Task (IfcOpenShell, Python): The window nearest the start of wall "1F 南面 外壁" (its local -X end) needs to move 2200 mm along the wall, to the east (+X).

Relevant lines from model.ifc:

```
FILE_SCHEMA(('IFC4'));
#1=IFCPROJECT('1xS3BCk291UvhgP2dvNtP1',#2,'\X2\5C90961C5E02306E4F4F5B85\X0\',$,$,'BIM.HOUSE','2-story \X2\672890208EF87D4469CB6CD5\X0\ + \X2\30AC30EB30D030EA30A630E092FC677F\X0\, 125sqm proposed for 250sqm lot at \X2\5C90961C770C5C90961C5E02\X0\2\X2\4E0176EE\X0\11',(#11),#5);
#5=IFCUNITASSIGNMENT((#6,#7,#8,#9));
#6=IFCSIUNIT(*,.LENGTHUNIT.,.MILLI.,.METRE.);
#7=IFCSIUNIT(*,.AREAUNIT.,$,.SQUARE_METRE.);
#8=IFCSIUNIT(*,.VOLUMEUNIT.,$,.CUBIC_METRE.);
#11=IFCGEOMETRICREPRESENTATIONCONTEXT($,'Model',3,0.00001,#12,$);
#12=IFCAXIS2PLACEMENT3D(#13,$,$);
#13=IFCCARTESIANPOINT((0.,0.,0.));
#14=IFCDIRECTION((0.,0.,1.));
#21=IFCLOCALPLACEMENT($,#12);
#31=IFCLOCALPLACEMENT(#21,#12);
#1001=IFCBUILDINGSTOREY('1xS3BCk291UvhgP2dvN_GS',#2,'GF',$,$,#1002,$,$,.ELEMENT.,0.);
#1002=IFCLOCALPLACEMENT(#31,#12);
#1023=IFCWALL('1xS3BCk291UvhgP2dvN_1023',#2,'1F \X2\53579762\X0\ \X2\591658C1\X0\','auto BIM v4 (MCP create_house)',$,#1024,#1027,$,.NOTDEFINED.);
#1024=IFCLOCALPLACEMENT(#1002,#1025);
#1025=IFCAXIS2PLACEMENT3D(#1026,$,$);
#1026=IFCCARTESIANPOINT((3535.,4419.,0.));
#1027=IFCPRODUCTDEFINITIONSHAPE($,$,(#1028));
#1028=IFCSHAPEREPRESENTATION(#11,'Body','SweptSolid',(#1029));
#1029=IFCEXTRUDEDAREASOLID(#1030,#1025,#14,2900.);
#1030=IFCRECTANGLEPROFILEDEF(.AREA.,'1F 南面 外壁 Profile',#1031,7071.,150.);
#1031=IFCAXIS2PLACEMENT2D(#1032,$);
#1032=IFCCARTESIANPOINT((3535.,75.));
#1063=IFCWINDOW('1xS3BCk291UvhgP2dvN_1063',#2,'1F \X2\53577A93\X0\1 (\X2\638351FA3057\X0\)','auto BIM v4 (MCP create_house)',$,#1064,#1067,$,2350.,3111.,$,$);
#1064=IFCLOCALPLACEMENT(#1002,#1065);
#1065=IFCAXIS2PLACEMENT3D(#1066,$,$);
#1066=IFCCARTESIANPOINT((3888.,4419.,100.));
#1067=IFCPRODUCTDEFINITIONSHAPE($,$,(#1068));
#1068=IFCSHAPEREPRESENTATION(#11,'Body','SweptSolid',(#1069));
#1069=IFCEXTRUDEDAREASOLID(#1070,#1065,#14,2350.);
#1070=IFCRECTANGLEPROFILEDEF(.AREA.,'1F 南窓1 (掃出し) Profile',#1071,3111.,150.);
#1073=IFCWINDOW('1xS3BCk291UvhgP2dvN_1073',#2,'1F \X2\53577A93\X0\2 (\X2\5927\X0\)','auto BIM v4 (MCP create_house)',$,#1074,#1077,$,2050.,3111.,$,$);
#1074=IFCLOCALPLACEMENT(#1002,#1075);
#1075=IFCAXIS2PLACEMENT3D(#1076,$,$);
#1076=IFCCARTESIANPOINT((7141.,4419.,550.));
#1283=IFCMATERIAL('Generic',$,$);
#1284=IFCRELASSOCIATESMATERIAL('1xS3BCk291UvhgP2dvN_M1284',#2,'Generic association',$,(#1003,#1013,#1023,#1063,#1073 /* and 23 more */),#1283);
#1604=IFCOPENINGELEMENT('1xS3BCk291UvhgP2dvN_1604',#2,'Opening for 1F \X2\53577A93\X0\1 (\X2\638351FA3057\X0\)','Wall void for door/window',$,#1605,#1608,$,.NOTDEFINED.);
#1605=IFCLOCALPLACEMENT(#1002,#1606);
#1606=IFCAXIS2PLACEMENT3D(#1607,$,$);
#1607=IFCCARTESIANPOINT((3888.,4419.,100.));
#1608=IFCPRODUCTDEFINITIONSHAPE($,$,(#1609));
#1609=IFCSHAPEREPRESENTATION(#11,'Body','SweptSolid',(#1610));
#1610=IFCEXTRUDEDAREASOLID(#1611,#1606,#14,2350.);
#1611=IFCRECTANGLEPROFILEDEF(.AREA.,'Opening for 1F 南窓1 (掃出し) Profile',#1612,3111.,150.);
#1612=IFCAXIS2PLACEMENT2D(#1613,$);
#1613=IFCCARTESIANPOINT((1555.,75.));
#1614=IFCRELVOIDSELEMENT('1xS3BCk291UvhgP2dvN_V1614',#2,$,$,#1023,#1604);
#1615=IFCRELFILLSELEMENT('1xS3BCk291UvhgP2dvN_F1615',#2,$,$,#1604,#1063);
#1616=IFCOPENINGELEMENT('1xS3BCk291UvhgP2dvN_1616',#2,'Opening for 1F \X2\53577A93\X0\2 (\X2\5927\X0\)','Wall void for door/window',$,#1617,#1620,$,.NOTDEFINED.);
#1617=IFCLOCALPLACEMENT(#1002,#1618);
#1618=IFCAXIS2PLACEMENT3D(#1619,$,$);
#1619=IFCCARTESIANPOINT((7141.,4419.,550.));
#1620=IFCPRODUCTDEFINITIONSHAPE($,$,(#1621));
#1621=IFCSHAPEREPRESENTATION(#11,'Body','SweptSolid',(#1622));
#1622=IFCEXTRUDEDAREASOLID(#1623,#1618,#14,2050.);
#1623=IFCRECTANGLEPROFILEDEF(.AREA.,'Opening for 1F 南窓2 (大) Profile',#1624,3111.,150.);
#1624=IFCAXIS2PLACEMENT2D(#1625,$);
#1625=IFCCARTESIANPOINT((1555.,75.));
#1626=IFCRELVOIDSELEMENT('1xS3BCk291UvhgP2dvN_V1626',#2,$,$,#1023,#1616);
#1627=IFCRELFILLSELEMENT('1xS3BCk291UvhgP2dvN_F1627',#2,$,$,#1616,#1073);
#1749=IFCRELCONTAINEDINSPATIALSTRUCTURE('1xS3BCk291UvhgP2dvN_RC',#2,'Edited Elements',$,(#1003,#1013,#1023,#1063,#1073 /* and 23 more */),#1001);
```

```python
import ifcopenshell
import ifcopenshell.api.geometry
import ifcopenshell.util.placement
import ifcopenshell.util.unit

model = ifcopenshell.open("model.ifc")
unit_scale = ifcopenshell.util.unit.calculate_unit_scale(model)

window = model.by_guid("1xS3BCk291UvhgP2dvN_1063")
opening = window.FillsVoids[0].RelatingOpeningElement
wall = opening.VoidsElements[0].RelatingBuildingElement

wall_matrix = ifcopenshell.util.placement.get_local_placement(wall.ObjectPlacement)
shift = wall_matrix[:3, 0] * 2.2 / unit_scale
before = ifcopenshell.util.placement.get_local_placement(window.ObjectPlacement)[:3, 3].copy()

# The window is not placed relative to its opening, so move both.
for product in (opening, window):
    matrix = ifcopenshell.util.placement.get_local_placement(product.ObjectPlacement)
    matrix[:3, 3] += shift
    ifcopenshell.api.geometry.edit_object_placement(model, product=product, matrix=matrix, is_si=False)

after = ifcopenshell.util.placement.get_local_placement(window.ObjectPlacement)[:3, 3]
print("window moved by", (after - before).round(3) + 0.0)

model.write("model_v2.ifc")
```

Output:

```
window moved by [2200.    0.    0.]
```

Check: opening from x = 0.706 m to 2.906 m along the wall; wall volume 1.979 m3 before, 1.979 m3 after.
